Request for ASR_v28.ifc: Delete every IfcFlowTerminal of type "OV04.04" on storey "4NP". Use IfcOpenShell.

First a look at what the model holds.

```python
import ifcopenshell
import ifcopenshell.util.element

model = ifcopenshell.open("ASR_v28.ifc")
print(model.schema)
storey = next(s for s in model.by_type("IfcBuildingStorey") if s.Name == "4NP")
terminals = [e for e in ifcopenshell.util.element.get_decomposition(storey) if e.is_a("IfcFlowTerminal")]
seen = {}
for e in terminals:
    element_type = ifcopenshell.util.element.get_type(e)
    name = element_type.Name if element_type not in (None, e) else None
    seen[name] = seen.get(name, 0) + 1
for name, count in sorted(seen.items(), key=str):
    print(count, "x", name)
```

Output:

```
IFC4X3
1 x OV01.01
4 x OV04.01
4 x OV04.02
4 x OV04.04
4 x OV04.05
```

```python
import ifcopenshell
import ifcopenshell.api.root
import ifcopenshell.util.element

model = ifcopenshell.open("ASR_v28.ifc")

storey = next(s for s in model.by_type("IfcBuildingStorey") if s.Name == "4NP")
terminals = [e for e in ifcopenshell.util.element.get_decomposition(storey) if e.is_a("IfcFlowTerminal")]
targets = [e for e in terminals if (t := ifcopenshell.util.element.get_type(e)) not in (None, e) and t.Name == "OV04.04"]

for e in targets:
    ifcopenshell.api.root.remove_product(model, product=e)
print(len(targets), "removed")

model.write("ASR_v28_rev.ifc")
```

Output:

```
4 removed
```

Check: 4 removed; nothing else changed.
